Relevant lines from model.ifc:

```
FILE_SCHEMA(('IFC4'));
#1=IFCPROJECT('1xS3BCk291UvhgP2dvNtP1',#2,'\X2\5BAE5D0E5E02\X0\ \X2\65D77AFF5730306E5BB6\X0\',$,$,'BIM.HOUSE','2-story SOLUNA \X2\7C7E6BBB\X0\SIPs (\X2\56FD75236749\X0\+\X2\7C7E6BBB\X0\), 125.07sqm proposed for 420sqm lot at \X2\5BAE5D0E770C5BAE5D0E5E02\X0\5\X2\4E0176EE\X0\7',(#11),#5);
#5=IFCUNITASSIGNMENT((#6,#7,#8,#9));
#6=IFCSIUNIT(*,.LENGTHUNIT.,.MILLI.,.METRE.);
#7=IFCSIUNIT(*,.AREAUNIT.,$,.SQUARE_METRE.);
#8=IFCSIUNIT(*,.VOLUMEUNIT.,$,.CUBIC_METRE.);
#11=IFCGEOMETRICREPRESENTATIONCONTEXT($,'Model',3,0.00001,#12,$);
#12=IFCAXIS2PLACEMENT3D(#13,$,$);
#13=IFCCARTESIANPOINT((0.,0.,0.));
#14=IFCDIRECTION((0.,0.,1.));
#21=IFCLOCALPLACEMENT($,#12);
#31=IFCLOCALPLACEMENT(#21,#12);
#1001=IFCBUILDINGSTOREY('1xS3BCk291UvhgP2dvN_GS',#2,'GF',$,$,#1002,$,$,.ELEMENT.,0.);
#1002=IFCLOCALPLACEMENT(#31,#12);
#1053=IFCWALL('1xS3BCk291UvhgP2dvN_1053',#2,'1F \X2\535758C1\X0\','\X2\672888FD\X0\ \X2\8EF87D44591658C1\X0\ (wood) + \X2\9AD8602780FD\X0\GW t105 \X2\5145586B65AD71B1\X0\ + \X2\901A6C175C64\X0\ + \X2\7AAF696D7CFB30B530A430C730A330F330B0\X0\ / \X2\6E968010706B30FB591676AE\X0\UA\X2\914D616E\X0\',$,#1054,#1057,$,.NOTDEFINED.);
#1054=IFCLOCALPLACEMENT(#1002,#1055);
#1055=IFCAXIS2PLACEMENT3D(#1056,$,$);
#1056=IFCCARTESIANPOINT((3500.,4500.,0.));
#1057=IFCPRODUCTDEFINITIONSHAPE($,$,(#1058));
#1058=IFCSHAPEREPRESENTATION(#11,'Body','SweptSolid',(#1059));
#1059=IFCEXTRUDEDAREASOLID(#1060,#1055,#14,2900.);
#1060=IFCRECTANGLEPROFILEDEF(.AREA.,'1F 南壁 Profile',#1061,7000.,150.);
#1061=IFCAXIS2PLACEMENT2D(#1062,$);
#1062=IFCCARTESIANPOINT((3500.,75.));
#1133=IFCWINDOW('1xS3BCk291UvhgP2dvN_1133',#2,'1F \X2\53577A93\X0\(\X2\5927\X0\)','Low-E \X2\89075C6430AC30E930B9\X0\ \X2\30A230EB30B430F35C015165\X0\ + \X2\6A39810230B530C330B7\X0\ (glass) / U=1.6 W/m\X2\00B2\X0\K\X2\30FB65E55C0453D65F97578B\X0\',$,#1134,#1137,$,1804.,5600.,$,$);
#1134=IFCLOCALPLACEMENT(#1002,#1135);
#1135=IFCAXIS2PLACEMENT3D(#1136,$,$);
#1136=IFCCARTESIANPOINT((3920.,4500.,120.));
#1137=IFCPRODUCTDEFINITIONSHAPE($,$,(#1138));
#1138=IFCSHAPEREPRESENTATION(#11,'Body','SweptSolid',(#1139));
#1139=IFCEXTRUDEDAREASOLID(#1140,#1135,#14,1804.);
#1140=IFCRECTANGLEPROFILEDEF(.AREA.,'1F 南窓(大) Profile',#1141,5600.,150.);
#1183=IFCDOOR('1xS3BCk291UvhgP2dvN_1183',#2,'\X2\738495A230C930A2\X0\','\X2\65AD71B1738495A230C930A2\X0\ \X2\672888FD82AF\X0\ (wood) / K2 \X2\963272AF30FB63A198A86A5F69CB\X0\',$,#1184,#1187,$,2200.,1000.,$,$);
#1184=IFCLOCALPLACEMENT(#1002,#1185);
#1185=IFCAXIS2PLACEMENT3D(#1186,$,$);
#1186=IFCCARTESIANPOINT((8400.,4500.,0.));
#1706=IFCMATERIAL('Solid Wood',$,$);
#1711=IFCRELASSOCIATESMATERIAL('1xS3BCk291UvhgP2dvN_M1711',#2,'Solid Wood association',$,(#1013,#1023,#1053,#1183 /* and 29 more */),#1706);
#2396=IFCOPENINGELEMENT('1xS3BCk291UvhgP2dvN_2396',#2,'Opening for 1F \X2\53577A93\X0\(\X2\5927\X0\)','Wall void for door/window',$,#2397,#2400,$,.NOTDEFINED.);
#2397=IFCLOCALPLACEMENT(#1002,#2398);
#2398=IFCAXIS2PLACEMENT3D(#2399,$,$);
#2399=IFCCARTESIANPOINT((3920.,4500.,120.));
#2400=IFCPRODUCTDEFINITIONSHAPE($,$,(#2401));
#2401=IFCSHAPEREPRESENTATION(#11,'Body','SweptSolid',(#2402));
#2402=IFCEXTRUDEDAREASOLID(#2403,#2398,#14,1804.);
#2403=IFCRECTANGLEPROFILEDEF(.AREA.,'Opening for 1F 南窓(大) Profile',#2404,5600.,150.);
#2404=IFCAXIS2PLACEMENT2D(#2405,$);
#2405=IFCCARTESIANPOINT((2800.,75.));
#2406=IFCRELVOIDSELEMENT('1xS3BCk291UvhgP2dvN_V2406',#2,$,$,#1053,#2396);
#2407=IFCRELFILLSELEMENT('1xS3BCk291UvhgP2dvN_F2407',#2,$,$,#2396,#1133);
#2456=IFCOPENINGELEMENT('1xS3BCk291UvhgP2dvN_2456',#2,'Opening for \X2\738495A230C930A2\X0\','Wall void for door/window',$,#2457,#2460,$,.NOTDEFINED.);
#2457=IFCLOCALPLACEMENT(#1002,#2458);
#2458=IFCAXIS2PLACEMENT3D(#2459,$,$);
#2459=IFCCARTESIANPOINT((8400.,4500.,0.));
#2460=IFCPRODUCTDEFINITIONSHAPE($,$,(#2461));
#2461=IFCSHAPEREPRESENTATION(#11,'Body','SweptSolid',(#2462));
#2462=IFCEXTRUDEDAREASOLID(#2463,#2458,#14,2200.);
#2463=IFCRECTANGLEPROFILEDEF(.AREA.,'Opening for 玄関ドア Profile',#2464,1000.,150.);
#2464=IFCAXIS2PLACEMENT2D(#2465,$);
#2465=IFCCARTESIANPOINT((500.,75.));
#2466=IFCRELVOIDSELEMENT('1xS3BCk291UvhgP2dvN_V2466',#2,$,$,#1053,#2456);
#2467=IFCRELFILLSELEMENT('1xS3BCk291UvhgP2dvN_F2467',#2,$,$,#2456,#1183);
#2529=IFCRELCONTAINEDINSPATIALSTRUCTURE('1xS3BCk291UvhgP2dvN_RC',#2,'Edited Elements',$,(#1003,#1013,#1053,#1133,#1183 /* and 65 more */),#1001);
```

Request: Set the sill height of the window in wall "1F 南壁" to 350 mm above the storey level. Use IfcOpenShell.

```python
import numpy as np
import ifcopenshell
import ifcopenshell.api.geometry
import ifcopenshell.geom
import ifcopenshell.util.element
import ifcopenshell.util.placement
import ifcopenshell.util.shape
import ifcopenshell.util.unit

model = ifcopenshell.open("model.ifc")
unit_scale = ifcopenshell.util.unit.calculate_unit_scale(model)

window = model.by_guid("1xS3BCk291UvhgP2dvN_1133")
opening = window.FillsVoids[0].RelatingOpeningElement
storey = ifcopenshell.util.element.get_container(window, ifc_class="IfcBuildingStorey")
level = ifcopenshell.util.placement.get_local_placement(storey.ObjectPlacement)[2, 3]

# The opening's origin need not be at the sill, so measure its lowest point.
shape = ifcopenshell.geom.create_shape(ifcopenshell.geom.settings(), opening)
bottom = ifcopenshell.util.shape.get_shape_bottom_elevation(shape, shape.geometry) / unit_scale
dz = level + 0.35 / unit_scale - bottom

shift = np.array([0.0, 0.0, dz])
# The window is not placed relative to its opening, so move both.
for product in (opening, window):
    matrix = ifcopenshell.util.placement.get_local_placement(product.ObjectPlacement)
    matrix[:3, 3] += shift
    ifcopenshell.api.geometry.edit_object_placement(model, product=product, matrix=matrix, is_si=False)

print(f"moved by {dz * unit_scale:+.3f} m")

model.write("model_updated.ifc")
```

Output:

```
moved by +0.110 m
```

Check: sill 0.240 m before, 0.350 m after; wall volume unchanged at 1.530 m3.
